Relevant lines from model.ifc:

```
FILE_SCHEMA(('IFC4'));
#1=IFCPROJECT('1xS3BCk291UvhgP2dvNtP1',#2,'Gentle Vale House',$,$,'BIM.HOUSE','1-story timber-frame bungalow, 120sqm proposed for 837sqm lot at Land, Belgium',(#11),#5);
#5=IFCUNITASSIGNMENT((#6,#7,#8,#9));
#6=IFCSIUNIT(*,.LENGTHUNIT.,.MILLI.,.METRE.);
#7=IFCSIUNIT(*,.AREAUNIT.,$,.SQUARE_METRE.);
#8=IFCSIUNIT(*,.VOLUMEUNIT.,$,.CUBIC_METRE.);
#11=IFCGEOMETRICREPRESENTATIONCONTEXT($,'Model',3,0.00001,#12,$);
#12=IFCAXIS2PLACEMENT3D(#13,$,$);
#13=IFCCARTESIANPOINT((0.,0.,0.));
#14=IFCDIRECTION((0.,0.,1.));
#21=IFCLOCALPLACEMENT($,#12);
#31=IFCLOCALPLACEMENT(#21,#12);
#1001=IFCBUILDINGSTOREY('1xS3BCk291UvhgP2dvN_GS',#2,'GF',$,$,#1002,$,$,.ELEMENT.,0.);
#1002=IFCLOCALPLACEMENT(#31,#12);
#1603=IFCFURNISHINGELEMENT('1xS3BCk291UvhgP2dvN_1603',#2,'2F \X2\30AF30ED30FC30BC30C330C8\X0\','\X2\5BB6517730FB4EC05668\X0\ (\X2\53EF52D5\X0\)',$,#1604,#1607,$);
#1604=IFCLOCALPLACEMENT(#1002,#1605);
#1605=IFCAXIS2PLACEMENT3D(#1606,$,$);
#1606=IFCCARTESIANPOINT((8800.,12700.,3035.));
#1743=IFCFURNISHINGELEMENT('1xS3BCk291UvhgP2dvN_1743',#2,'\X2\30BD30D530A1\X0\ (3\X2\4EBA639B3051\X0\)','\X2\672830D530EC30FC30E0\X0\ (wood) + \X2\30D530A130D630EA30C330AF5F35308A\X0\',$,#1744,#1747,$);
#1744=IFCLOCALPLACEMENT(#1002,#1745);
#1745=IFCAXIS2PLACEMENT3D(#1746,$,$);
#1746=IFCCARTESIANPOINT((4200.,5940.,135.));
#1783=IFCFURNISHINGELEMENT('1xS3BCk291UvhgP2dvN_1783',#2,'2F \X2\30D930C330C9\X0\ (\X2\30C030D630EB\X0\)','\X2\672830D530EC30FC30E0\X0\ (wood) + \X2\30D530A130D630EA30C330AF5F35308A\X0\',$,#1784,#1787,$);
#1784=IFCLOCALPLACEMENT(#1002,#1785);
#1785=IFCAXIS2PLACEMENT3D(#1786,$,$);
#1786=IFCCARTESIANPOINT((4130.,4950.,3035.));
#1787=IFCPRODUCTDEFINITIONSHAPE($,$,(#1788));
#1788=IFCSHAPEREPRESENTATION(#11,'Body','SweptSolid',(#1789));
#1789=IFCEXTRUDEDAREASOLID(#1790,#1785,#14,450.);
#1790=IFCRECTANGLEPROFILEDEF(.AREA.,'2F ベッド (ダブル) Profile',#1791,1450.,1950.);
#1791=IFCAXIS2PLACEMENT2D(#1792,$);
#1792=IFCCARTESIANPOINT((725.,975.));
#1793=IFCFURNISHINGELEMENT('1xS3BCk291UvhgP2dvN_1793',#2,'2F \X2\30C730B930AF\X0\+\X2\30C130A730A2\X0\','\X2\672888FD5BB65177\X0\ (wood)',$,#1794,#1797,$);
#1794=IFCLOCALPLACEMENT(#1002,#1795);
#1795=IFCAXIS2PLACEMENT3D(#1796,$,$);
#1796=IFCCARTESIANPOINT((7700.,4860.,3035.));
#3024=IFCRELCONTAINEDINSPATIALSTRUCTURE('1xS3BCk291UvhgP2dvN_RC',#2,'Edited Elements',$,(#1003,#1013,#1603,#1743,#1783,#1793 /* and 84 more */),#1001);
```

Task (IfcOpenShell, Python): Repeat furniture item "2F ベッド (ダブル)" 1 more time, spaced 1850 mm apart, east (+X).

```python
import numpy as np
import ifcopenshell
import ifcopenshell.api.geometry
import ifcopenshell.api.root
import ifcopenshell.util.element
import ifcopenshell.util.placement

model = ifcopenshell.open("model.ifc")


def reuse_history(source, copy):
    """copy_class also copies each property set's owner history, people and application; keep the originals."""
    for rel in copy.IsDefinedBy:
        if rel.is_a("IfcRelDefinesByProperties") and (history := rel.RelatingPropertyDefinition.OwnerHistory):
            rel.RelatingPropertyDefinition.OwnerHistory = source.OwnerHistory
            ifcopenshell.util.element.remove_deep2(model, history)


source = model.by_id(1783)
base = ifcopenshell.util.placement.get_local_placement(source.ObjectPlacement)
step = np.array([1.0, 0.0, 0.0]) * 1850.0

for i in range(1, 2):
    copy = ifcopenshell.api.root.copy_class(model, product=source)
    copy.Representation = ifcopenshell.util.element.copy_deep(
        model, source.Representation, exclude=["IfcGeometricRepresentationContext", "IfcRepresentationMap"]
    )
    reuse_history(source, copy)
    matrix = base.copy()
    matrix[:3, 3] += i * step
    print("added at", matrix[:3, 3].round(3) + 0.0)
    ifcopenshell.api.geometry.edit_object_placement(model, product=copy, matrix=matrix, is_si=False)

model.write("model_edited.ifc")
```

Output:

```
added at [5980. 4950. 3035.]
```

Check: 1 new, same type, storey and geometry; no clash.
